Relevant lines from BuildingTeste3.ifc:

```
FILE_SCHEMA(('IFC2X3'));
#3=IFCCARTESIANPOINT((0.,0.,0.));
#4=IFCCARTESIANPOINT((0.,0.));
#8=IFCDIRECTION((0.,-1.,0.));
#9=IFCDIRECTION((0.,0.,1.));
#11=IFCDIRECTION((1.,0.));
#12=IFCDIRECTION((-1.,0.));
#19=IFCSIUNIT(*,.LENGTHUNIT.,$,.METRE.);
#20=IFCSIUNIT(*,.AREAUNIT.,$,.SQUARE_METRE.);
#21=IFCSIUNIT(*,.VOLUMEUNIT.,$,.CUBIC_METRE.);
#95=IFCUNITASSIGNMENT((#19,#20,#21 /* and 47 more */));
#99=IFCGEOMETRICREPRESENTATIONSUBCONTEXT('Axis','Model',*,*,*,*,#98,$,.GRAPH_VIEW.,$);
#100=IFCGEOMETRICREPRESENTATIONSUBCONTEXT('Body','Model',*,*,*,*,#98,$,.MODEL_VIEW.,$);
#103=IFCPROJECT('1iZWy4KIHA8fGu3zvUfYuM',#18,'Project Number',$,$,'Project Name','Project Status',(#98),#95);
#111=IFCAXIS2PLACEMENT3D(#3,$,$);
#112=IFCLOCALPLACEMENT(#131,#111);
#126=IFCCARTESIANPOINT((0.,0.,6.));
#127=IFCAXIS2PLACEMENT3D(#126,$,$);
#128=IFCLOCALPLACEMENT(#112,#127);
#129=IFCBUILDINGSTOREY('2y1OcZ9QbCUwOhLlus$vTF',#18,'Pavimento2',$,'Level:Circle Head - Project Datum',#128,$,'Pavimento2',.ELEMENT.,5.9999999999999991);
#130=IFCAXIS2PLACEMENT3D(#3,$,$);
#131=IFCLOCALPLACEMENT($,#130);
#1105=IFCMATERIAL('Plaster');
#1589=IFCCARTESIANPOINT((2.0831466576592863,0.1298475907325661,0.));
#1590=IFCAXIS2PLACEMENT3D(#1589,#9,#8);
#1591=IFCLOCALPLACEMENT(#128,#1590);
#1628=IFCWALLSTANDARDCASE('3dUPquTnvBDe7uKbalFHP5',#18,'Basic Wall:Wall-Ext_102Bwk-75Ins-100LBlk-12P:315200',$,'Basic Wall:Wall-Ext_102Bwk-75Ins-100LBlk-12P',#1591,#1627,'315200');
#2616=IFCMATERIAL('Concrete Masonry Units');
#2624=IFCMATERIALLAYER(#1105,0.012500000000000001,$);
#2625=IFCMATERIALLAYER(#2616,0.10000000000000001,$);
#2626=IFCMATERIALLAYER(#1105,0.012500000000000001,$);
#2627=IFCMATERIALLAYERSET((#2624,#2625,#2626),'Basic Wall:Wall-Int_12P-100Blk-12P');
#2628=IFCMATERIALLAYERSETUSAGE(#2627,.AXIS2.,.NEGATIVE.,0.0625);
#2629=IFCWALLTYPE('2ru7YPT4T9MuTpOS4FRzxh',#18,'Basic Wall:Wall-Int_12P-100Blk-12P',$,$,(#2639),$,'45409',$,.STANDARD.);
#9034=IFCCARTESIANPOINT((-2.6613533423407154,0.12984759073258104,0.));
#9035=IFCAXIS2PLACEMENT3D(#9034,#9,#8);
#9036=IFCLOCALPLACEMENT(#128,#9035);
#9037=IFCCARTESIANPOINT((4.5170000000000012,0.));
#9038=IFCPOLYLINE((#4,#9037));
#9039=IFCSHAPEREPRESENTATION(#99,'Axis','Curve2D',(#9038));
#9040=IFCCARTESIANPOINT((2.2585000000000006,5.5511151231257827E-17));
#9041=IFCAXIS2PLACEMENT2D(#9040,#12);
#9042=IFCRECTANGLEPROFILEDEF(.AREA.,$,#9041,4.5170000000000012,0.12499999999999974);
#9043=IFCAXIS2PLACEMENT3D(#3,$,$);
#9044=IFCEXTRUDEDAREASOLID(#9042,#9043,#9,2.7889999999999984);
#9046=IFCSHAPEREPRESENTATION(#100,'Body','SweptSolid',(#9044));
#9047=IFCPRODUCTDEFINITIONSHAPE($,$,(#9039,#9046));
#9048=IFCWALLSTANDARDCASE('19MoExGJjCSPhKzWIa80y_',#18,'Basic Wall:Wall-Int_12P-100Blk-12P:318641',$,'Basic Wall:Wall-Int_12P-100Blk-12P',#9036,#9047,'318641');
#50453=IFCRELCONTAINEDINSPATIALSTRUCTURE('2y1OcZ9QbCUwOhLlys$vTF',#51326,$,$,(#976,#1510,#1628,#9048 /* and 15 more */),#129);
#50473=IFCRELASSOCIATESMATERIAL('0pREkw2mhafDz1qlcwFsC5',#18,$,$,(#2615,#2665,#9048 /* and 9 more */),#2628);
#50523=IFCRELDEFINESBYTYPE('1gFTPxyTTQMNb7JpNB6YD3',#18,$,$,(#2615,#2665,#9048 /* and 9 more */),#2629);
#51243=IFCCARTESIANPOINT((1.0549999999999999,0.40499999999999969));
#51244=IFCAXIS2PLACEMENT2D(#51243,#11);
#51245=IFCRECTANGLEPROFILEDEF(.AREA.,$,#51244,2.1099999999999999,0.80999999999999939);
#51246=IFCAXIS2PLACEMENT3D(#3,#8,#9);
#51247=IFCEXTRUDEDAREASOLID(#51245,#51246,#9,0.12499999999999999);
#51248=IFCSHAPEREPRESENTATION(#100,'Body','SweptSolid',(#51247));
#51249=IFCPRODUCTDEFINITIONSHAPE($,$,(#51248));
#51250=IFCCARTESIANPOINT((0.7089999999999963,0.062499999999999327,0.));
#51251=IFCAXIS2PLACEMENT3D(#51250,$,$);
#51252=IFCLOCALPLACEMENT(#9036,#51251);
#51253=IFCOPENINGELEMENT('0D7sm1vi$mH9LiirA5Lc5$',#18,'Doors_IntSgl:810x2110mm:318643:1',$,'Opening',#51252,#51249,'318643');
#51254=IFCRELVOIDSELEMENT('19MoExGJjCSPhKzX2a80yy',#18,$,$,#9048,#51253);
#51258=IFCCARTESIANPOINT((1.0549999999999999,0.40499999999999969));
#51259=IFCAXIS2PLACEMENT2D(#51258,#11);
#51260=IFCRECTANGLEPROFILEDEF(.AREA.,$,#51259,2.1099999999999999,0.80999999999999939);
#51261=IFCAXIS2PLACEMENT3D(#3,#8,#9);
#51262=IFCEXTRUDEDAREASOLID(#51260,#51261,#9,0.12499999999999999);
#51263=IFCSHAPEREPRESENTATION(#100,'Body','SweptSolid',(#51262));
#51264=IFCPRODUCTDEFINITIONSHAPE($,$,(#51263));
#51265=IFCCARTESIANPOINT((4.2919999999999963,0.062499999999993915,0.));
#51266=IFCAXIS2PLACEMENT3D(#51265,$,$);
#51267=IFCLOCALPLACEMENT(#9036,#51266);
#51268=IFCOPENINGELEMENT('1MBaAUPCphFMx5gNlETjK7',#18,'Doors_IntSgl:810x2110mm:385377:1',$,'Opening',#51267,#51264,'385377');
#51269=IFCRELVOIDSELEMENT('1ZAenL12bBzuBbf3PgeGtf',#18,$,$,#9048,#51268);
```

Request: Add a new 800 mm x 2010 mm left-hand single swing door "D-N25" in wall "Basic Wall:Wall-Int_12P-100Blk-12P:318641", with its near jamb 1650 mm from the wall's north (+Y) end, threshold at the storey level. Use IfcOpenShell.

```python
import numpy as np
import ifcopenshell
import ifcopenshell.api.feature
import ifcopenshell.api.geometry
import ifcopenshell.api.root
import ifcopenshell.api.spatial
import ifcopenshell.api.type
import ifcopenshell.geom
import ifcopenshell.util.element
import ifcopenshell.util.placement
import ifcopenshell.util.representation
import ifcopenshell.util.shape
import ifcopenshell.util.unit

model = ifcopenshell.open("BuildingTeste3.ifc")
unit_scale = ifcopenshell.util.unit.calculate_unit_scale(model)
settings = ifcopenshell.geom.settings()


def volume(element):
    """Net volume in cubic metres, openings subtracted."""
    shape = ifcopenshell.geom.create_shape(settings, element)
    return ifcopenshell.util.shape.get_volume(shape.geometry)


wall = model.by_id(9048)
storey = ifcopenshell.util.element.get_container(wall, ifc_class="IfcBuildingStorey")
context = ifcopenshell.util.representation.get_context(model, "Model", "Body", "MODEL_VIEW")
before = volume(wall)

width, height, from_end, sill = 0.8, 2.01, 1.65, 0.0  # metres

# The wall runs along its own X axis, and the end named is its -X end.
wall_shape = ifcopenshell.geom.create_shape(settings, wall)
x, y, z = ifcopenshell.util.shape.get_vertices(wall_shape.geometry).T
start = x.min() + from_end
face, thickness = float(y.min()), float(y.max() - y.min())
wall_matrix = ifcopenshell.util.placement.get_local_placement(wall.ObjectPlacement)
level = ifcopenshell.util.placement.get_local_placement(storey.ObjectPlacement)[2, 3]


def in_wall(x, y):
    """Placement at x, y metres in the wall's axes, at sill height."""
    matrix = wall_matrix.copy()
    matrix[:, 3] = wall_matrix @ np.array([x / unit_scale, y / unit_scale, 0.0, 1.0])
    matrix[2, 3] = level + sill / unit_scale
    return matrix


# Opening: a box that overshoots both wall faces by 50 mm.
opening = ifcopenshell.api.root.create_entity(model, ifc_class="IfcOpeningElement")
box = ifcopenshell.api.geometry.add_wall_representation(
    model, context=context, length=width, height=height, thickness=thickness + 0.1
)
ifcopenshell.api.geometry.assign_representation(model, product=opening, representation=box)
ifcopenshell.api.geometry.edit_object_placement(model, product=opening, matrix=in_wall(start, face - 0.05), is_si=False)
ifcopenshell.api.feature.add_feature(model, feature=opening, element=wall)

door = ifcopenshell.api.root.create_entity(model, ifc_class="IfcDoor", name="D-N25")
door.OverallWidth, door.OverallHeight = width / unit_scale, height / unit_scale
body = ifcopenshell.api.geometry.add_door_representation(
    model,
    context=context,
    overall_width=door.OverallWidth,
    overall_height=door.OverallHeight,
    operation_type="SINGLE_SWING_LEFT",
    lining_properties={"LiningDepth": thickness / unit_scale, "ThresholdDepth": thickness / unit_scale},
)
ifcopenshell.api.geometry.assign_representation(model, product=door, representation=body)
ifcopenshell.api.spatial.assign_container(model, products=[door], relating_structure=storey)
fills = ifcopenshell.api.feature.add_filling(model, opening=opening, element=door)
fills.OwnerHistory = door.OwnerHistory  # required in IFC2X3

# IFC2X3 keeps the operation on the door style.
style = ifcopenshell.api.root.create_entity(model, ifc_class="IfcDoorStyle", name="D-N25")
style.OperationType, style.ConstructionType = "SINGLE_SWING_LEFT", "NOTDEFINED"
style.ParameterTakesPrecedence = style.Sizeable = False
ifcopenshell.api.type.assign_type(model, related_objects=[door], relating_type=style)

# The lining spans the wall, so the door starts at the wall face.
ifcopenshell.api.geometry.edit_object_placement(model, product=door, matrix=in_wall(start, face), is_si=False)

after = volume(wall)

print(f"wall volume {before:.3f} -> {after:.3f} m3")

model.write("BuildingTeste3-out.ifc")
```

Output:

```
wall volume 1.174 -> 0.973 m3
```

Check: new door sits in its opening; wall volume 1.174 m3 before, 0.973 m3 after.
